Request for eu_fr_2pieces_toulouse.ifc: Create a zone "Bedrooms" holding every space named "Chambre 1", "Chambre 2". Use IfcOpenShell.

First a look at what the model holds.

```python
import ifcopenshell

model = ifcopenshell.open("eu_fr_2pieces_toulouse.ifc")
print(model.schema)
seen = {}
for space in model.by_type("IfcSpace"):
    seen[space.LongName] = seen.get(space.LongName, 0) + 1
for name, count in sorted(seen.items(), key=str):
    print(count, "x", name)
print("zones:", [z.Name for z in model.by_type("IfcZone")][:20])
```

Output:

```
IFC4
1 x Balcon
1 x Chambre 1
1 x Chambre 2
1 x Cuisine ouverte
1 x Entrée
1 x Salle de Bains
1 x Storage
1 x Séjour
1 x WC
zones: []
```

```python
import ifcopenshell
import ifcopenshell.api.group
import ifcopenshell.api.root

model = ifcopenshell.open("eu_fr_2pieces_toulouse.ifc")

names = {"Chambre 1", "Chambre 2"}
spaces = [s for s in model.by_type("IfcSpace") if s.LongName in names]

zone = ifcopenshell.api.root.create_entity(model, ifc_class="IfcZone", name="Bedrooms")
ifcopenshell.api.group.assign_group(model, products=spaces, group=zone)
print(len(spaces), "spaces in", zone.Name)

model.write("eu_fr_2pieces_toulouse_updated.ifc")
```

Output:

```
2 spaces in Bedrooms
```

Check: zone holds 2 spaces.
